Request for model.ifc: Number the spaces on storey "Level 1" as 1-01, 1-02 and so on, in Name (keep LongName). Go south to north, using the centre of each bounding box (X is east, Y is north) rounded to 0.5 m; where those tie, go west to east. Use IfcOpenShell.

First a look at what the model holds.

```python
import ifcopenshell
import ifcopenshell.util.element
import ifcopenshell.util.placement

model = ifcopenshell.open("model.ifc")
print(model.schema)
storey = next(s for s in model.by_type("IfcBuildingStorey") if s.Name == "Level 1")
spaces = [e for e in ifcopenshell.util.element.get_decomposition(storey) if e.is_a("IfcSpace")]
for e in sorted(spaces, key=lambda e: e.id()):
    origin = ifcopenshell.util.placement.get_local_placement(e.ObjectPlacement)[:3, 3]
    print(e.id(), e.Name, e.LongName, origin.round(2) + 0.0, sep=" | ")
```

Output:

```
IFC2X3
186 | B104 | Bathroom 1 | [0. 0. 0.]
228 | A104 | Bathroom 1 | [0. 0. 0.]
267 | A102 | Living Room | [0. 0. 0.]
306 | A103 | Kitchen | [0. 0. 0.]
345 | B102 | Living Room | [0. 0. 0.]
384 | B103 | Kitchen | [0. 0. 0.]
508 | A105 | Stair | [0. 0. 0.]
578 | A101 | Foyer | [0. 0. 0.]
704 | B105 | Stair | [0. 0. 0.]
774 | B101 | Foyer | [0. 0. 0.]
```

```python
import ifcopenshell
import ifcopenshell.geom
import ifcopenshell.util.element
import ifcopenshell.util.shape

model = ifcopenshell.open("model.ifc")
settings = ifcopenshell.geom.settings()
settings.set("use-world-coords", True)


def centre(element):
    shape = ifcopenshell.geom.create_shape(settings, element)
    return ifcopenshell.util.shape.get_bbox_centroid(shape.geometry)


storey = next(s for s in model.by_type("IfcBuildingStorey") if s.Name == "Level 1")
spaces = [e for e in ifcopenshell.util.element.get_decomposition(storey) if e.is_a("IfcSpace")]

# Insertion points can sit at a corner or the storey origin, so sort by the geometry (in metres).
centres = {e: centre(e) for e in spaces}
spaces.sort(key=lambda e: (round(centres[e][1] / 0.5), centres[e][0]))

for i, e in enumerate(spaces, start=1):
    number = f"1-{i:02d}"
    e.Name = number
    print(e.id(), number)

model.write("model_rev.ifc")
```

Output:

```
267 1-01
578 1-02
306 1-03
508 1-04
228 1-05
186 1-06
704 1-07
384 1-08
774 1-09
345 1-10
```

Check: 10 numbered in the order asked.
